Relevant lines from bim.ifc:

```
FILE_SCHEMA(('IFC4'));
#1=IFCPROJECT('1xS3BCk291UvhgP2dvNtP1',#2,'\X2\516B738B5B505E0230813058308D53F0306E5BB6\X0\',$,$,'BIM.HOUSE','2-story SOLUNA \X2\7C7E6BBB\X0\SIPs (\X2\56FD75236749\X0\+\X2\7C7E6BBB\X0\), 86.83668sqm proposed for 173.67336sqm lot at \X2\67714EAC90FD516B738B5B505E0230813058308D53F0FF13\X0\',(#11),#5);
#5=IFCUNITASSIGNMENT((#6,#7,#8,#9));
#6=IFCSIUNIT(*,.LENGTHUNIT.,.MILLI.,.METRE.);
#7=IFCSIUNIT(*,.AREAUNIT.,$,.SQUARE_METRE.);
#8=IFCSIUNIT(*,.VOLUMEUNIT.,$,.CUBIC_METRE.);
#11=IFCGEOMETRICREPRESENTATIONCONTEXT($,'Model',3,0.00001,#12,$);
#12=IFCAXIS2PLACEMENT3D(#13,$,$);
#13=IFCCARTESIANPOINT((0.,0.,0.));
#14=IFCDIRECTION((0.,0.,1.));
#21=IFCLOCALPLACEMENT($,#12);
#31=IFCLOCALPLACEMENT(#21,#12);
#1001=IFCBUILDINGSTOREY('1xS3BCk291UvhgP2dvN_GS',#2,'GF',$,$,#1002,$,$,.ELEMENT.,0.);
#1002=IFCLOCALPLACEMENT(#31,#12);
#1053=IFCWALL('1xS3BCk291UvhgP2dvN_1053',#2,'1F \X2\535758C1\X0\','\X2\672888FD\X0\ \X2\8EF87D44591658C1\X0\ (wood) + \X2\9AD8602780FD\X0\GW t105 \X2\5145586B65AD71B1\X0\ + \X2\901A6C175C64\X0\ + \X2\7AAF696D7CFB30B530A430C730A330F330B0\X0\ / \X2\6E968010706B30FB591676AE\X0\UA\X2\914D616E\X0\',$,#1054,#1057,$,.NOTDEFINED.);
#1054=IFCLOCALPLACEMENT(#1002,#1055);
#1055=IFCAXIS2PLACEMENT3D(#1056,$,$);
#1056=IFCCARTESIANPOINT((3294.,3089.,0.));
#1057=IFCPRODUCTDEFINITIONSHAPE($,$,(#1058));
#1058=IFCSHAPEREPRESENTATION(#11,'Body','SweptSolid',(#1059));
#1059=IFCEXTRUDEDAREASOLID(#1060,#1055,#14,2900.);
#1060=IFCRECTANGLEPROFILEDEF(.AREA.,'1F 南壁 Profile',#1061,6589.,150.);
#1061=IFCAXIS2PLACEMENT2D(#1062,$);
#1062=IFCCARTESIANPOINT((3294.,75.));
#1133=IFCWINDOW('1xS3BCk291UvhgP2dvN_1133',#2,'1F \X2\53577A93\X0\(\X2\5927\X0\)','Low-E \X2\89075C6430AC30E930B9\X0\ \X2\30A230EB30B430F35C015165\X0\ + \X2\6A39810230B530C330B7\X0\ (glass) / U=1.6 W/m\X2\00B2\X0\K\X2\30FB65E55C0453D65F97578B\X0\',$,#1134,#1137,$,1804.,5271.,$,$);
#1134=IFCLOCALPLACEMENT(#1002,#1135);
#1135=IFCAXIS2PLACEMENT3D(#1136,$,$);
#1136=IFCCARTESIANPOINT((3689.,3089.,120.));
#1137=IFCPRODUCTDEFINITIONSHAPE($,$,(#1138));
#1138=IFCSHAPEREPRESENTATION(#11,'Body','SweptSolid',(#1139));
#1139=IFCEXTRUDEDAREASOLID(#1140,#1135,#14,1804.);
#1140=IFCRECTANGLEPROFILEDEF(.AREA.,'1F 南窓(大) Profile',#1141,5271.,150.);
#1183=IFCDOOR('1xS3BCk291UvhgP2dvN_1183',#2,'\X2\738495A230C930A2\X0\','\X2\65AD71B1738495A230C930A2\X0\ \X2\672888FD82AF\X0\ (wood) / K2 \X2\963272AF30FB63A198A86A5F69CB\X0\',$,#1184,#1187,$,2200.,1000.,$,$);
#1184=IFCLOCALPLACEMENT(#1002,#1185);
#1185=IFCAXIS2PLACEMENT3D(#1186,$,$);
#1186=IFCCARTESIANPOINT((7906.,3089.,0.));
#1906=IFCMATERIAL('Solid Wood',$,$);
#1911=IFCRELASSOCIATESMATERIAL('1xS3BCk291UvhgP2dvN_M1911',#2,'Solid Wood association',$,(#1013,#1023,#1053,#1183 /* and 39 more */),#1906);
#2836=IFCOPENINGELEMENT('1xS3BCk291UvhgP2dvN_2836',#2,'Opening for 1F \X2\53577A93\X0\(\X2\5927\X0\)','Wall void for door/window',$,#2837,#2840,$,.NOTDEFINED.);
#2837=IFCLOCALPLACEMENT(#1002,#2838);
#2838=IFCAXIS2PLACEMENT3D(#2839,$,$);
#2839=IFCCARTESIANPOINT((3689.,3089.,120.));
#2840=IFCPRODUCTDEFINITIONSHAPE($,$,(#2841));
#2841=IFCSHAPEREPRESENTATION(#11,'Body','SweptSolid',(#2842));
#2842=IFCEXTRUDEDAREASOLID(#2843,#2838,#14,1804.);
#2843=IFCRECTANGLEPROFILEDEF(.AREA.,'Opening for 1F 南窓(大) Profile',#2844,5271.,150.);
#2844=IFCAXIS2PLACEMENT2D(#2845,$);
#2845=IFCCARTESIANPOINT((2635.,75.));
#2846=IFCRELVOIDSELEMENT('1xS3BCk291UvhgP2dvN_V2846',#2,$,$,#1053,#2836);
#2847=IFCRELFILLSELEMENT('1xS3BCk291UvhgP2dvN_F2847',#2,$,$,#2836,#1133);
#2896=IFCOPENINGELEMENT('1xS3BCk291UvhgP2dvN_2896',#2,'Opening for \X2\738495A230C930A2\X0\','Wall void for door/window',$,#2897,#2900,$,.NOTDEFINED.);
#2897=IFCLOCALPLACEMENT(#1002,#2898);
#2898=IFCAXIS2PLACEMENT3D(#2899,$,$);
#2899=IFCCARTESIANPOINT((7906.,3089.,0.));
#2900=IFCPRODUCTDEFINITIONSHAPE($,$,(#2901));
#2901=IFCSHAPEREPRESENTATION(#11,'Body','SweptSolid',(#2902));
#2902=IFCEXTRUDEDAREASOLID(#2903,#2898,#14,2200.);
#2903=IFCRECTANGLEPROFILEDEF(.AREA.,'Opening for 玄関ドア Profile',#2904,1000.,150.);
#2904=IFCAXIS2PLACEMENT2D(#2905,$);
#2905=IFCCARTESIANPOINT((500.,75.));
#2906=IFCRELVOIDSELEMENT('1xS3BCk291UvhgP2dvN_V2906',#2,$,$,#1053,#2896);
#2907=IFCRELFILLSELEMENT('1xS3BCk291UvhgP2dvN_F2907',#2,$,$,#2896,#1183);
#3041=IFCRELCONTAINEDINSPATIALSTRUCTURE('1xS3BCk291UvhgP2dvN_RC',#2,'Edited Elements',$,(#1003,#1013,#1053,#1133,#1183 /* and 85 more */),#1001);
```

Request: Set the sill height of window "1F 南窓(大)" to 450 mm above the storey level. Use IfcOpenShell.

```python
import numpy as np
import ifcopenshell
import ifcopenshell.api.geometry
import ifcopenshell.geom
import ifcopenshell.util.element
import ifcopenshell.util.placement
import ifcopenshell.util.shape
import ifcopenshell.util.unit

model = ifcopenshell.open("bim.ifc")
unit_scale = ifcopenshell.util.unit.calculate_unit_scale(model)

window = model.by_guid("1xS3BCk291UvhgP2dvN_1133")
opening = window.FillsVoids[0].RelatingOpeningElement
storey = ifcopenshell.util.element.get_container(window, ifc_class="IfcBuildingStorey")
level = ifcopenshell.util.placement.get_local_placement(storey.ObjectPlacement)[2, 3]

# The opening's origin need not be at the sill, so measure its lowest point.
shape = ifcopenshell.geom.create_shape(ifcopenshell.geom.settings(), opening)
bottom = ifcopenshell.util.shape.get_shape_bottom_elevation(shape, shape.geometry) / unit_scale
dz = level + 0.45 / unit_scale - bottom

shift = np.array([0.0, 0.0, dz])
# The window is not placed relative to its opening, so move both.
for product in (opening, window):
    matrix = ifcopenshell.util.placement.get_local_placement(product.ObjectPlacement)
    matrix[:3, 3] += shift
    ifcopenshell.api.geometry.edit_object_placement(model, product=product, matrix=matrix, is_si=False)

print(f"moved by {dz * unit_scale:+.3f} m")

model.write("bim_edited.ifc")
```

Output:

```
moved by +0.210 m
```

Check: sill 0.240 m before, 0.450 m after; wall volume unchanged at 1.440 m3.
